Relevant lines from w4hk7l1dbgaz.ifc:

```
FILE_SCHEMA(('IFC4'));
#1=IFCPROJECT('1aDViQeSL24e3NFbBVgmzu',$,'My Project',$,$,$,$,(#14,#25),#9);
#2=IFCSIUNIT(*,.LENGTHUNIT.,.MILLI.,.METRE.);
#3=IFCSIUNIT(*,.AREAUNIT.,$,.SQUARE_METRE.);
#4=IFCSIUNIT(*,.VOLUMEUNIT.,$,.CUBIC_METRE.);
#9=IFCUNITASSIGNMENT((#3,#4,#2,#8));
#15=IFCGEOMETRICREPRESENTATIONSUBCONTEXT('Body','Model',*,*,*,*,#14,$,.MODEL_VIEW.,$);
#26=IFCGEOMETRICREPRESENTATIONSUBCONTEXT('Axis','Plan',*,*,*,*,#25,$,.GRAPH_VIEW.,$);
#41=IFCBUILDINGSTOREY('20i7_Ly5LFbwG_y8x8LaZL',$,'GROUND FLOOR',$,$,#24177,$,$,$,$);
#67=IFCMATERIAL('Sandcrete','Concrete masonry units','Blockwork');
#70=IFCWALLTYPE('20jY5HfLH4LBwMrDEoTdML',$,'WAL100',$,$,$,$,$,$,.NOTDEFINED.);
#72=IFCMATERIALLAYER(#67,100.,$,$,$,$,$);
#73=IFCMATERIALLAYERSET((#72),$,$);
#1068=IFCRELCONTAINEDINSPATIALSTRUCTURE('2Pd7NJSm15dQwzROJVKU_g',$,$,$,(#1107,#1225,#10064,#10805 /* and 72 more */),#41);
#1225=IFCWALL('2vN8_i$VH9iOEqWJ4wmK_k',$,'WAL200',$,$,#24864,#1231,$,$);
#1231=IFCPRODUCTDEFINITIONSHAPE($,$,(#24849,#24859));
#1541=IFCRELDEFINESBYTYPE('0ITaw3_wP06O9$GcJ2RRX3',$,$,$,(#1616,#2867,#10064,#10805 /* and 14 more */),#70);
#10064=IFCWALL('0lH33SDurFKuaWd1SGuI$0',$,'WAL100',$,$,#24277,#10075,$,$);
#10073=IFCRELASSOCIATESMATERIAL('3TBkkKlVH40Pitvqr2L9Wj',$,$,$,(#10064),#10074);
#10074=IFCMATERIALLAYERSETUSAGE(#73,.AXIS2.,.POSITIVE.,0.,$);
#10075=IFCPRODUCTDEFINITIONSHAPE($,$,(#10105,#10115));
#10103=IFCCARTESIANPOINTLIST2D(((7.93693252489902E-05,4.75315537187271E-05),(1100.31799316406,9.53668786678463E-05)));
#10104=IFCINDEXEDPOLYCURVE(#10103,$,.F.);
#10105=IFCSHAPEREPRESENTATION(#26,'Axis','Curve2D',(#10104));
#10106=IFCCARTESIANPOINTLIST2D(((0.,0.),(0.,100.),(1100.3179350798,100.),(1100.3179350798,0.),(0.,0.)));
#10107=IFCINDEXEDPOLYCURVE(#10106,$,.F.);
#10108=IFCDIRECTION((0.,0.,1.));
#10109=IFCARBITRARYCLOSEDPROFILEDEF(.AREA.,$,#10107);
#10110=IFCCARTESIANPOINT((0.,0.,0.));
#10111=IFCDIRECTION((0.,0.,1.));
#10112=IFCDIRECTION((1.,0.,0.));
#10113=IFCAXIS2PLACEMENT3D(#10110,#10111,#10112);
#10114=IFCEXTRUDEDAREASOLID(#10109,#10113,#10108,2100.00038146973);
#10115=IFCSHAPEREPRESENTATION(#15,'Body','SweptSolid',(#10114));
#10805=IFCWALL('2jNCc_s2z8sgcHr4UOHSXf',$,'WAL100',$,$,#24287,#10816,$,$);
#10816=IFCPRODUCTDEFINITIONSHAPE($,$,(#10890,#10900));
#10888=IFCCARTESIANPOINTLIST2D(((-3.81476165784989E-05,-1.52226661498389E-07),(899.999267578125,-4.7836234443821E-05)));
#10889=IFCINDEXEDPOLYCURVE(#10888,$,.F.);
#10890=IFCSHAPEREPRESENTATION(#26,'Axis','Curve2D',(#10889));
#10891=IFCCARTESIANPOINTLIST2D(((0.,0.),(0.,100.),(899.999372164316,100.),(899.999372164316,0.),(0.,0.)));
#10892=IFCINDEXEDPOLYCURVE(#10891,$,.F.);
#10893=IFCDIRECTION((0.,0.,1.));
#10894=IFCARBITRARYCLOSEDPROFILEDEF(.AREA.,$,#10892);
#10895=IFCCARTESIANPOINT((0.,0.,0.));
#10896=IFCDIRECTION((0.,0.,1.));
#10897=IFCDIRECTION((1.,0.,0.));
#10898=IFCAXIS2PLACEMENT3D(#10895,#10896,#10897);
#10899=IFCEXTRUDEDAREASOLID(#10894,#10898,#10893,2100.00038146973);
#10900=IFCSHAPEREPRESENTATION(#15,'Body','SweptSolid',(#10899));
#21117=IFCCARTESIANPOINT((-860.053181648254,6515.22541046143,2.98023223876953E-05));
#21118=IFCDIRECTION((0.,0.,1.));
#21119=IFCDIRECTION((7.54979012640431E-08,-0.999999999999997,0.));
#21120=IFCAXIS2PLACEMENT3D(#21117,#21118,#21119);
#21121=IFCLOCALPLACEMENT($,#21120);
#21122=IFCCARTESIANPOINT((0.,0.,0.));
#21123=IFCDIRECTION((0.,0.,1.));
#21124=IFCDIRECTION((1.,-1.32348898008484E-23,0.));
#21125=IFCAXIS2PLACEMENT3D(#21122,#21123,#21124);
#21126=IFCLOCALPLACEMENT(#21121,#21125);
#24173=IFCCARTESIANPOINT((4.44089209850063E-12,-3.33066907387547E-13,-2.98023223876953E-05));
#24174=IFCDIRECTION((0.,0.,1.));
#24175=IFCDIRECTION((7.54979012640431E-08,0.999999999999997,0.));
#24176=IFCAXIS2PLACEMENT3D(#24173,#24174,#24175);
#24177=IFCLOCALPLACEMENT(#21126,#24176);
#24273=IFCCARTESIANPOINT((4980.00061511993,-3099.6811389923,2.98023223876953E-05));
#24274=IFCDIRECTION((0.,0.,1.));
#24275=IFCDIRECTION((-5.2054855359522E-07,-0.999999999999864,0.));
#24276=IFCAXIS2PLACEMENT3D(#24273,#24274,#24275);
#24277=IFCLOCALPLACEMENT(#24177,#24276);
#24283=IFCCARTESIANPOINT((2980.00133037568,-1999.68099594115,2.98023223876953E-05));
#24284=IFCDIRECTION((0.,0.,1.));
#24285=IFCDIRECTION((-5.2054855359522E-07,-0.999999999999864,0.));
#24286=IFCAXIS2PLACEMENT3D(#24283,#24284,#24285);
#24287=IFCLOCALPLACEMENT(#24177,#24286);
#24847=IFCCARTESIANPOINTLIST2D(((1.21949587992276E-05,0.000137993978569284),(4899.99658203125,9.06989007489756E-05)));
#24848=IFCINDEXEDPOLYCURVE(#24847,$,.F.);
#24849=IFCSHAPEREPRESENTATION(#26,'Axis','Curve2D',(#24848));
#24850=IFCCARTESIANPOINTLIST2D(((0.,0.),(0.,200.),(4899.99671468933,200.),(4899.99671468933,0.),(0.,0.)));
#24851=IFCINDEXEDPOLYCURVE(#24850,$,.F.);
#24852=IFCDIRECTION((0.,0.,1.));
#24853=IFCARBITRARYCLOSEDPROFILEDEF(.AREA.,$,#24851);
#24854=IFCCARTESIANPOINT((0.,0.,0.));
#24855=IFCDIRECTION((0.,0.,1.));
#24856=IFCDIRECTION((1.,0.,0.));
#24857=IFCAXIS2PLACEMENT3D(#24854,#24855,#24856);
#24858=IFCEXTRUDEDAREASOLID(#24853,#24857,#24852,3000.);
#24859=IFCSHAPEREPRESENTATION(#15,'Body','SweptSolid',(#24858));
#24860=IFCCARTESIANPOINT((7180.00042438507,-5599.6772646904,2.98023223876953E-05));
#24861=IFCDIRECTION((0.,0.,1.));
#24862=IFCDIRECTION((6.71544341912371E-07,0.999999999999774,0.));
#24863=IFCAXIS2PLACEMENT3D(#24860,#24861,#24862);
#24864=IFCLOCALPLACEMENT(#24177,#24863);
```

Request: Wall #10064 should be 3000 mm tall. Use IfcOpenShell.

```python
import ifcopenshell
import ifcopenshell.geom
import ifcopenshell.util.representation
import ifcopenshell.util.shape
import ifcopenshell.util.unit

model = ifcopenshell.open("w4hk7l1dbgaz.ifc")
unit_scale = ifcopenshell.util.unit.calculate_unit_scale(model)
settings = ifcopenshell.geom.settings()


def volume(element):
    """Net volume in cubic metres, openings subtracted."""
    shape = ifcopenshell.geom.create_shape(settings, element)
    return ifcopenshell.util.shape.get_volume(shape.geometry)


wall = model.by_id(10064)
before = volume(wall)

body = ifcopenshell.util.representation.get_representation(wall, "Model", "Body")
solid = body.Items[0]
old_height = solid.Depth
solid.Depth = 3 / unit_scale
after = volume(wall)

print(f"height {old_height:g} -> {solid.Depth:g}, volume {before:.3f} -> {after:.3f} m3")

model.write("w4hk7l1dbgaz_updated.ifc")
```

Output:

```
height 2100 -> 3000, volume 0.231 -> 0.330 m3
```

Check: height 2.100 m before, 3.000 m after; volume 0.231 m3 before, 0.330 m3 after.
